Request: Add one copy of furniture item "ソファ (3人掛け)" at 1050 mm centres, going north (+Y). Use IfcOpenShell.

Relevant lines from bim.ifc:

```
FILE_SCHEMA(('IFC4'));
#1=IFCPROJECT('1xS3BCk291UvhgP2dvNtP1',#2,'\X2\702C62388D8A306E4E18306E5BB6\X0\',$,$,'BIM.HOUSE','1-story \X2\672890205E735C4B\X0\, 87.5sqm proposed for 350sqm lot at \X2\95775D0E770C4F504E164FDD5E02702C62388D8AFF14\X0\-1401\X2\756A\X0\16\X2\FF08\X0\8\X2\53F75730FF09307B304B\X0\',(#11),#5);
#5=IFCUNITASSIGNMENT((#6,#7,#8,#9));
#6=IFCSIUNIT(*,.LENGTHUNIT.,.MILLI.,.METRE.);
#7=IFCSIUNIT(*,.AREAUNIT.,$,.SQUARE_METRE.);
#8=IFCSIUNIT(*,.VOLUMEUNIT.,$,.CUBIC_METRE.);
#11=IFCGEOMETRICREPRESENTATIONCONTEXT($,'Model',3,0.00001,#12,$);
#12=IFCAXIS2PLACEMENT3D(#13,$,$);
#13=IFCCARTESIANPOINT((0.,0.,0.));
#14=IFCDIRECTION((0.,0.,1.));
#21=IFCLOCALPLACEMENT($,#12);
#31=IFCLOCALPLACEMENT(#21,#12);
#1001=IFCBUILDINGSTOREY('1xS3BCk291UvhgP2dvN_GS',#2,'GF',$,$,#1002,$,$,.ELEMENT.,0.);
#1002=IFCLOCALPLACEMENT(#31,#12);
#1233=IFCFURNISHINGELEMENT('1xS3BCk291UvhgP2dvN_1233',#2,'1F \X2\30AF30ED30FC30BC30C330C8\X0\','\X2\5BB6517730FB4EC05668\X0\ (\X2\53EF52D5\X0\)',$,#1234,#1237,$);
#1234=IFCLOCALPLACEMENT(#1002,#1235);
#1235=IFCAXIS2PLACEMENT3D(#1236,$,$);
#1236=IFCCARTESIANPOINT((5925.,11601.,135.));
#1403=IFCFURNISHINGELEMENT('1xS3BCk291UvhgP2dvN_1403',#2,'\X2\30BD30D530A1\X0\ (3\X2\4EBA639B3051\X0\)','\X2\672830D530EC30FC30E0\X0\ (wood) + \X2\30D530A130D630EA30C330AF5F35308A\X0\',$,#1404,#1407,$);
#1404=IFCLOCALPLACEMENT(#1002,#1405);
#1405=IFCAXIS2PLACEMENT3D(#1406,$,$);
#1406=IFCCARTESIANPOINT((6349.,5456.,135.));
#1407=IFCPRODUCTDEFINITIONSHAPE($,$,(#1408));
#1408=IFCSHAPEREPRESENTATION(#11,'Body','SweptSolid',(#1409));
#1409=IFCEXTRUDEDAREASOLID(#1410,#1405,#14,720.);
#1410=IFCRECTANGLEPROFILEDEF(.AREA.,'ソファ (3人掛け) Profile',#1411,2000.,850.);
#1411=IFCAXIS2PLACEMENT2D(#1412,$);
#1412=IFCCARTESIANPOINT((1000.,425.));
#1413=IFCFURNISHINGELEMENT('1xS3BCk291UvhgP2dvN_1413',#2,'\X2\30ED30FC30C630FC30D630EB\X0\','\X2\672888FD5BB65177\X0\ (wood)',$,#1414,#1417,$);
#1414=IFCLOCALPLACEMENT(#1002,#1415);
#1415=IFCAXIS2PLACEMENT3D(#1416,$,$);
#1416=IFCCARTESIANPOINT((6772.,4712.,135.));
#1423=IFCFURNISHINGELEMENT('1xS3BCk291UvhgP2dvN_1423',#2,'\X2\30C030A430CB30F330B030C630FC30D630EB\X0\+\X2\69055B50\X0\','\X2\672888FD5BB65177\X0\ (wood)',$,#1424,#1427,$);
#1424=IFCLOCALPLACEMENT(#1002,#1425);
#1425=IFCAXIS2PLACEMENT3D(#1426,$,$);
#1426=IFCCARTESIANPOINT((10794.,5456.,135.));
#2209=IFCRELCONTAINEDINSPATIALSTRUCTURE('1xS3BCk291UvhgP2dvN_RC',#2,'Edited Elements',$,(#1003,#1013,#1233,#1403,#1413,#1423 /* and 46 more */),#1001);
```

```python
import numpy as np
import ifcopenshell
import ifcopenshell.api.geometry
import ifcopenshell.api.root
import ifcopenshell.util.element
import ifcopenshell.util.placement
import ifcopenshell.util.unit

model = ifcopenshell.open("bim.ifc")
unit_scale = ifcopenshell.util.unit.calculate_unit_scale(model)


def reuse_history(source, copy):
    """copy_class also copies each property set's owner history, people and application; keep the originals."""
    for rel in copy.IsDefinedBy:
        if rel.is_a("IfcRelDefinesByProperties") and (history := rel.RelatingPropertyDefinition.OwnerHistory):
            rel.RelatingPropertyDefinition.OwnerHistory = source.OwnerHistory
            ifcopenshell.util.element.remove_deep2(model, history)


source = model.by_id(1403)
base = ifcopenshell.util.placement.get_local_placement(source.ObjectPlacement)
step = np.array([0.0, 1.0, 0.0]) * 1.05 / unit_scale

for i in range(1, 2):
    copy = ifcopenshell.api.root.copy_class(model, product=source)
    copy.Representation = ifcopenshell.util.element.copy_deep(
        model, source.Representation, exclude=["IfcGeometricRepresentationContext", "IfcRepresentationMap"]
    )
    reuse_history(source, copy)
    matrix = base.copy()
    matrix[:3, 3] += i * step
    print("added at", matrix[:3, 3].round(3) + 0.0)
    ifcopenshell.api.geometry.edit_object_placement(model, product=copy, matrix=matrix, is_si=False)

model.write("bim_rev.ifc")
```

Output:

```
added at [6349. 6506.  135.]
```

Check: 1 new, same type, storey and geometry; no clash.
